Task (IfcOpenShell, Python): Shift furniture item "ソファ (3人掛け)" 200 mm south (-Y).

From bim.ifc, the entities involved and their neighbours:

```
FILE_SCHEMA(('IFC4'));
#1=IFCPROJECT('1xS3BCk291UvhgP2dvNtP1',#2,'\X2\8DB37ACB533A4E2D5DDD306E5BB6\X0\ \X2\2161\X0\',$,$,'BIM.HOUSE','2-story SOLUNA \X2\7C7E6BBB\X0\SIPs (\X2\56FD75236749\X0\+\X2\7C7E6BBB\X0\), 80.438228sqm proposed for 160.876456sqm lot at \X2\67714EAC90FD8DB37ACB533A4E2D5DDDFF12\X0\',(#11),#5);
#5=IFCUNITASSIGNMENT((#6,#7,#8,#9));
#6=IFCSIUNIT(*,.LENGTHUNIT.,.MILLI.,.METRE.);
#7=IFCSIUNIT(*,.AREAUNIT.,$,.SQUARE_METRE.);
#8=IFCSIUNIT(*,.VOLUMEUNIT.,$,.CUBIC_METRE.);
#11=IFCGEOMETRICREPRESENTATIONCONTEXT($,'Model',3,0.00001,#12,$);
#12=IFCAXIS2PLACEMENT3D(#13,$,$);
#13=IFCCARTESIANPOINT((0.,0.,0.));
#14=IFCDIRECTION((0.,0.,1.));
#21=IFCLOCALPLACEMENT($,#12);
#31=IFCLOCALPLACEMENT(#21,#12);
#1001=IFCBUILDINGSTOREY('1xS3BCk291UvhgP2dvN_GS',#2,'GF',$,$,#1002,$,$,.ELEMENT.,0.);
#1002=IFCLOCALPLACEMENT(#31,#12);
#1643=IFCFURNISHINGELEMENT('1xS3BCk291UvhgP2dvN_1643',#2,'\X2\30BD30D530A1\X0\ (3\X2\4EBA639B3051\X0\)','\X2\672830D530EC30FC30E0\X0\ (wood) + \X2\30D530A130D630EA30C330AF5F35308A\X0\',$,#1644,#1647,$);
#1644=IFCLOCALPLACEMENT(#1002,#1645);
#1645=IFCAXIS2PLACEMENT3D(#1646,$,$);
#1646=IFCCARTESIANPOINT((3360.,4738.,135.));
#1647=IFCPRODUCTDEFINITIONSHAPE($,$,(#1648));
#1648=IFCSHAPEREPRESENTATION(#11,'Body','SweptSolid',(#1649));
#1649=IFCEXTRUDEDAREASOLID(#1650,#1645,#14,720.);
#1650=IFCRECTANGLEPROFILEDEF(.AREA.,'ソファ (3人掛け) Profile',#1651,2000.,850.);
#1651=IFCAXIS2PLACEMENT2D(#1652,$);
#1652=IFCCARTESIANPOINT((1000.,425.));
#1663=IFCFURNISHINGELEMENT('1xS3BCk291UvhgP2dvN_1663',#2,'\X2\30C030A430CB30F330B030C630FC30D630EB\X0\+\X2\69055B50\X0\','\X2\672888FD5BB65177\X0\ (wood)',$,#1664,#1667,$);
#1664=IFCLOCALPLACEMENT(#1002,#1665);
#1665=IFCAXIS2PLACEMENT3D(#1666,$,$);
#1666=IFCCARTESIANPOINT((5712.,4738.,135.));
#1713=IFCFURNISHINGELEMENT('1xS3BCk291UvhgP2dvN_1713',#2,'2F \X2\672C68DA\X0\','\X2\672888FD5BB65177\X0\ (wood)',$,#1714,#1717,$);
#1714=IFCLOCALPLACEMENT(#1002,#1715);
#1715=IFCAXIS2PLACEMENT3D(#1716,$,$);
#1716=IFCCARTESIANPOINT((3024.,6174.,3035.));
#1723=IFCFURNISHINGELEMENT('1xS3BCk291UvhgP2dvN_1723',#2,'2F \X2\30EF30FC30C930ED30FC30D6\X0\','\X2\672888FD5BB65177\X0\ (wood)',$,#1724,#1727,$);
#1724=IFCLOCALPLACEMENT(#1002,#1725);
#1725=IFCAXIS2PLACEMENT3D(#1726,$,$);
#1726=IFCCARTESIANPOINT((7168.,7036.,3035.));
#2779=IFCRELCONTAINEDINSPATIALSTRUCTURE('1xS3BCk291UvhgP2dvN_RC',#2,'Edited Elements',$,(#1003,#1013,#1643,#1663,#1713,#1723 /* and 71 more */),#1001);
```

```python
import ifcopenshell
import ifcopenshell.api.geometry
import ifcopenshell.util.placement
import ifcopenshell.util.unit

model = ifcopenshell.open("bim.ifc")
unit_scale = ifcopenshell.util.unit.calculate_unit_scale(model)

item = model.by_id(1643)
matrix = ifcopenshell.util.placement.get_local_placement(item.ObjectPlacement)
matrix[1, 3] -= 0.2 / unit_scale
ifcopenshell.api.geometry.edit_object_placement(model, product=item, matrix=matrix, is_si=False)

print(ifcopenshell.util.placement.get_local_placement(item.ObjectPlacement).round(3) + 0.0)

model.write("bim_v2.ifc")
```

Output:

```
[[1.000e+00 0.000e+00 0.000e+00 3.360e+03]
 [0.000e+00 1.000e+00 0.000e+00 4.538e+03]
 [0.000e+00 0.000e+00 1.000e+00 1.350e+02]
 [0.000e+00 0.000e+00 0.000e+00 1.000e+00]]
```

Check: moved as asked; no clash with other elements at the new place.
